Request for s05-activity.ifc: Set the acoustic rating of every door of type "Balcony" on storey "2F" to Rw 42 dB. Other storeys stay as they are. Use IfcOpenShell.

First a look at what the model holds.

```python
import ifcopenshell
import ifcopenshell.util.element

model = ifcopenshell.open("s05-activity.ifc")
print(model.schema)
storey = next(s for s in model.by_type("IfcBuildingStorey") if s.Name == "2F")
doors = [e for e in ifcopenshell.util.element.get_decomposition(storey) if e.is_a("IfcDoor")]
seen = {}
for e in doors:
    element_type = ifcopenshell.util.element.get_type(e)
    key = (element_type.Name if element_type != e and element_type else None, ifcopenshell.util.element.get_pset(e, "Pset_DoorCommon", "AcousticRating"))
    seen[key] = seen.get(key, 0) + 1
for (name, value), count in sorted(seen.items(), key=str):
    print(count, "x", name, "|", value)
```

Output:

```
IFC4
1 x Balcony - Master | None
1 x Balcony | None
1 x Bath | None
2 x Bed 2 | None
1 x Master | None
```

```python
import ifcopenshell
import ifcopenshell.api.pset
import ifcopenshell.util.element

model = ifcopenshell.open("s05-activity.ifc")

storey = next(s for s in model.by_type("IfcBuildingStorey") if s.Name == "2F")
doors = [e for e in ifcopenshell.util.element.get_decomposition(storey) if e.is_a("IfcDoor")]

count = 0
for e in doors:
    element_type = ifcopenshell.util.element.get_type(e)
    if element_type in (None, e) or element_type.Name != "Balcony":
        continue
    # add_pset returns the element's existing set when there is one.
    pset = ifcopenshell.api.pset.add_pset(model, product=e, name="Pset_DoorCommon")
    ifcopenshell.api.pset.edit_pset(model, pset=pset, properties={"AcousticRating": "Rw 42 dB"})
    count += 1

print(count, "doors updated")

model.write("s05-activity_updated.ifc")
```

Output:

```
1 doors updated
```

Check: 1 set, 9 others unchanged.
